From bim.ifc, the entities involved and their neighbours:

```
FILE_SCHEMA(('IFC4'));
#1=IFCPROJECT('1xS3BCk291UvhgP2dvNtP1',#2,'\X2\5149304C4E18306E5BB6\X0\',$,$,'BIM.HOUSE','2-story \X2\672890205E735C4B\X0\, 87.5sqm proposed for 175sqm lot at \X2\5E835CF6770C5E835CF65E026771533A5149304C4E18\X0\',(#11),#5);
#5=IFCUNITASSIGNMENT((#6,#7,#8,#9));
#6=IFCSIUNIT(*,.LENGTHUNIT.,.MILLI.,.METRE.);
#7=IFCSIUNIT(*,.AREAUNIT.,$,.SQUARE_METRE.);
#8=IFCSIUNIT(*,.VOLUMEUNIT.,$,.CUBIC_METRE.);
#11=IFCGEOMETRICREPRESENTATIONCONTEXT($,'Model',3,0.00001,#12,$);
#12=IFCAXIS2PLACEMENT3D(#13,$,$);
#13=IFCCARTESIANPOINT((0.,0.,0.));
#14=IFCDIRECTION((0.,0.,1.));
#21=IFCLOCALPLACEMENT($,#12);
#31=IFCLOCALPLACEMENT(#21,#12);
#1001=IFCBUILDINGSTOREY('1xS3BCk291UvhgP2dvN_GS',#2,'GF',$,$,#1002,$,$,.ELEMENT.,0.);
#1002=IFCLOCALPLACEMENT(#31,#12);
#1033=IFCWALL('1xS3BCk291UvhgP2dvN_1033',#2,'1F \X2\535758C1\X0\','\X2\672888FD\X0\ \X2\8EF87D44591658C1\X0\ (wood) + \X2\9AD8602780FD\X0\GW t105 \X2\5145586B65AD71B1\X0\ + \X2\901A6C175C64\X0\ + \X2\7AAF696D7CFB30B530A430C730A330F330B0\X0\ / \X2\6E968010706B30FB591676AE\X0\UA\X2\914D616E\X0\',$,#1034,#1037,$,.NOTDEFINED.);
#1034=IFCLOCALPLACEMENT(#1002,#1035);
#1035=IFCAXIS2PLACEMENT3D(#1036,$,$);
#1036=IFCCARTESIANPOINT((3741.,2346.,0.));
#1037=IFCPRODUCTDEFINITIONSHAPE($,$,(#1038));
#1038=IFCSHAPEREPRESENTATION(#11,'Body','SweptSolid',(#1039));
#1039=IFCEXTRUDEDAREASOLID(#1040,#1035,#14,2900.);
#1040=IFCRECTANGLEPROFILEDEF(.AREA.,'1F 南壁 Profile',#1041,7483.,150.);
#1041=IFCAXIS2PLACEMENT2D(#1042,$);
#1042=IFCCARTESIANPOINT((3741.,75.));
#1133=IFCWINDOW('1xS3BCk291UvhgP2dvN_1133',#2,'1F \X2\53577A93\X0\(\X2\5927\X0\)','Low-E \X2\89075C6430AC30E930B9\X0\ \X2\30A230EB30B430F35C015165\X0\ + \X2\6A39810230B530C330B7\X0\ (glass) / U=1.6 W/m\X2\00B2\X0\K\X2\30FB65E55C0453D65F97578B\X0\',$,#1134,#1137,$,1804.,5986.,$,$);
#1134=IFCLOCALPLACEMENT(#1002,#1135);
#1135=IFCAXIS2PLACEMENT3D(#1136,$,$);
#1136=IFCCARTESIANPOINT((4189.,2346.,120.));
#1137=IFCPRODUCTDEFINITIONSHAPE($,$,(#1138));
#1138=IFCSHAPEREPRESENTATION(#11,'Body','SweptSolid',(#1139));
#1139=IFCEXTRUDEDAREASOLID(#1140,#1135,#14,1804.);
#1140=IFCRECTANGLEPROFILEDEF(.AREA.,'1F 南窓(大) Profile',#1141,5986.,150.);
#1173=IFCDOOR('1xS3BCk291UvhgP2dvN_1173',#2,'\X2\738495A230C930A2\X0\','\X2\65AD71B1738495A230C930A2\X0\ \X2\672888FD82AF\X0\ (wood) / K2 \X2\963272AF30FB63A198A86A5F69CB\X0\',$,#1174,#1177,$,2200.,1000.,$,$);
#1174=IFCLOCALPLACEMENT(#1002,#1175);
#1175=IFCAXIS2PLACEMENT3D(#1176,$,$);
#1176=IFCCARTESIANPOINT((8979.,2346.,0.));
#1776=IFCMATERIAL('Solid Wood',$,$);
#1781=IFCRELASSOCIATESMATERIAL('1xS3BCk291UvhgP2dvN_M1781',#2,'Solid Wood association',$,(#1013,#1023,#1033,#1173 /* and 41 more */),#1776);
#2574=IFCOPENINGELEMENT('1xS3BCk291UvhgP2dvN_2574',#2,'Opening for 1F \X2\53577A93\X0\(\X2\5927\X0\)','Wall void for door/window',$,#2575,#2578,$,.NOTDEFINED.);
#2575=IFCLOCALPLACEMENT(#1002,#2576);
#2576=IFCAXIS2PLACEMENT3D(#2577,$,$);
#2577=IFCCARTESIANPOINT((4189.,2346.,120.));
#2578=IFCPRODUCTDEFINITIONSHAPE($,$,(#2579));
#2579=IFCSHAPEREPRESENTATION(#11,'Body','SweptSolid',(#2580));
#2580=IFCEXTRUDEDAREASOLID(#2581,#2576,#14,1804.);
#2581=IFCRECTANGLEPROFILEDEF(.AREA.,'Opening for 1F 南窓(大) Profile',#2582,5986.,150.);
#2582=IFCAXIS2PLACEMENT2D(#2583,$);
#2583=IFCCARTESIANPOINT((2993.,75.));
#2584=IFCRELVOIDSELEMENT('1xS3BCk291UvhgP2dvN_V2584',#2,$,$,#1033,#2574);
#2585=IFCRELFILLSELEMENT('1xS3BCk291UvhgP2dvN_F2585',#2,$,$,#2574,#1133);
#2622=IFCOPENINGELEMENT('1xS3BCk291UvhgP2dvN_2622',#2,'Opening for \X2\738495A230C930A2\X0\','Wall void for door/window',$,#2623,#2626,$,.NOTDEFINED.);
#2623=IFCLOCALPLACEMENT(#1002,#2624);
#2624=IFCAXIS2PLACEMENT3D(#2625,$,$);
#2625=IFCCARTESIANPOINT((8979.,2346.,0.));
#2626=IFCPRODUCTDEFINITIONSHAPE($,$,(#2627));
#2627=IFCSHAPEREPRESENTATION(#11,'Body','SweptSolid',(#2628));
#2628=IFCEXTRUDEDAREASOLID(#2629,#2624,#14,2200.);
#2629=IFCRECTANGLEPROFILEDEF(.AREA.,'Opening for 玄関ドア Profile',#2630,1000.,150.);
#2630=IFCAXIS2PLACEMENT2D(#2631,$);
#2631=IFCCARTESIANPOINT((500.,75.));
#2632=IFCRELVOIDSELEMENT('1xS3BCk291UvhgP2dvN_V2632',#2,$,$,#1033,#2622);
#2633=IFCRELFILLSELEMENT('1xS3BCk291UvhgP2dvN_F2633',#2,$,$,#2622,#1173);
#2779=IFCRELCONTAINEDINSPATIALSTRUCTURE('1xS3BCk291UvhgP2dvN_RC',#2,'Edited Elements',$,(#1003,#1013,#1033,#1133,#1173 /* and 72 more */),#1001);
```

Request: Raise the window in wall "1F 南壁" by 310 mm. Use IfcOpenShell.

```python
import numpy as np
import ifcopenshell
import ifcopenshell.api.geometry
import ifcopenshell.util.placement
import ifcopenshell.util.unit

model = ifcopenshell.open("bim.ifc")
unit_scale = ifcopenshell.util.unit.calculate_unit_scale(model)

window = model.by_guid("1xS3BCk291UvhgP2dvN_1133")
opening = window.FillsVoids[0].RelatingOpeningElement
dz = 310.0

shift = np.array([0.0, 0.0, dz])
# The window is not placed relative to its opening, so move both.
for product in (opening, window):
    matrix = ifcopenshell.util.placement.get_local_placement(product.ObjectPlacement)
    matrix[:3, 3] += shift
    ifcopenshell.api.geometry.edit_object_placement(model, product=product, matrix=matrix, is_si=False)

print(f"moved by {dz * unit_scale:+.3f} m")

model.write("bim_rev.ifc")
```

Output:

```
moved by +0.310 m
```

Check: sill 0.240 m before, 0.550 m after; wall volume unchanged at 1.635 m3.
